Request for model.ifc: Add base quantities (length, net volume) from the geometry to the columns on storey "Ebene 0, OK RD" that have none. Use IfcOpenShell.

First a look at what the model holds.

```python
import ifcopenshell
import ifcopenshell.util.element
import ifcopenshell.util.unit

model = ifcopenshell.open("model.ifc")
print(model.schema)
for unit_type in ("LENGTHUNIT", "AREAUNIT", "VOLUMEUNIT"):
    print(unit_type, ifcopenshell.util.unit.calculate_unit_scale(model, unit_type))
storey = next(s for s in model.by_type("IfcBuildingStorey") if s.Name == "Ebene 0, OK RD")
columns = [e for e in ifcopenshell.util.element.get_decomposition(storey) if e.is_a("IfcColumn")]
for e in sorted(columns, key=lambda e: e.id()):
    print(e.id(), e.is_a(), e.Name, list(ifcopenshell.util.element.get_psets(e, qtos_only=True)), sep=" | ")
```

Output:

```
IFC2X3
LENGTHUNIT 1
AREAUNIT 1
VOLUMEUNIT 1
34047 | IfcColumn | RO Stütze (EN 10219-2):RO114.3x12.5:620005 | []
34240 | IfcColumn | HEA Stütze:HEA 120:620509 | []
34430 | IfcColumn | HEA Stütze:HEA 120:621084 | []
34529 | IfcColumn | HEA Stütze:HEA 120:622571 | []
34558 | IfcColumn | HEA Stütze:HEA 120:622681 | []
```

```python
import ifcopenshell
import ifcopenshell.api.pset
import ifcopenshell.geom
import ifcopenshell.util.element
import ifcopenshell.util.shape
import ifcopenshell.util.unit

model = ifcopenshell.open("model.ifc")
unit_scale = ifcopenshell.util.unit.calculate_unit_scale(model)
volume_scale = ifcopenshell.util.unit.calculate_unit_scale(model, "VOLUMEUNIT")
settings = ifcopenshell.geom.settings()

storey = next(s for s in model.by_type("IfcBuildingStorey") if s.Name == "Ebene 0, OK RD")
columns = [e for e in ifcopenshell.util.element.get_decomposition(storey) if e.is_a("IfcColumn")]

for e in sorted(columns, key=lambda e: e.id()):
    if ifcopenshell.util.element.get_psets(e, qtos_only=True, should_inherit=False):
        continue
    # Geometry comes back in metres, in the element's own axes.
    shape = ifcopenshell.geom.create_shape(settings, e)
    values = {
        "Length": ifcopenshell.util.shape.get_z(shape.geometry) / unit_scale,
        "NetVolume": ifcopenshell.util.shape.get_volume(shape.geometry) / volume_scale,
    }
    qto = ifcopenshell.api.pset.add_qto(model, product=e, name="BaseQuantities")
    ifcopenshell.api.pset.edit_qto(model, qto=qto, properties=values)
    print(e.id(), {k: round(v, 3) for k, v in values.items()})

model.write("model_updated.ifc")
```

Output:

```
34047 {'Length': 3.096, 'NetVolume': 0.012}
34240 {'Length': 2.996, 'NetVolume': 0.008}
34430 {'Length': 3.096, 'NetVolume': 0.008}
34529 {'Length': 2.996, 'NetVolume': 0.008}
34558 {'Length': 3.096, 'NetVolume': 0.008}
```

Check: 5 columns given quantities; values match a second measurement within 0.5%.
